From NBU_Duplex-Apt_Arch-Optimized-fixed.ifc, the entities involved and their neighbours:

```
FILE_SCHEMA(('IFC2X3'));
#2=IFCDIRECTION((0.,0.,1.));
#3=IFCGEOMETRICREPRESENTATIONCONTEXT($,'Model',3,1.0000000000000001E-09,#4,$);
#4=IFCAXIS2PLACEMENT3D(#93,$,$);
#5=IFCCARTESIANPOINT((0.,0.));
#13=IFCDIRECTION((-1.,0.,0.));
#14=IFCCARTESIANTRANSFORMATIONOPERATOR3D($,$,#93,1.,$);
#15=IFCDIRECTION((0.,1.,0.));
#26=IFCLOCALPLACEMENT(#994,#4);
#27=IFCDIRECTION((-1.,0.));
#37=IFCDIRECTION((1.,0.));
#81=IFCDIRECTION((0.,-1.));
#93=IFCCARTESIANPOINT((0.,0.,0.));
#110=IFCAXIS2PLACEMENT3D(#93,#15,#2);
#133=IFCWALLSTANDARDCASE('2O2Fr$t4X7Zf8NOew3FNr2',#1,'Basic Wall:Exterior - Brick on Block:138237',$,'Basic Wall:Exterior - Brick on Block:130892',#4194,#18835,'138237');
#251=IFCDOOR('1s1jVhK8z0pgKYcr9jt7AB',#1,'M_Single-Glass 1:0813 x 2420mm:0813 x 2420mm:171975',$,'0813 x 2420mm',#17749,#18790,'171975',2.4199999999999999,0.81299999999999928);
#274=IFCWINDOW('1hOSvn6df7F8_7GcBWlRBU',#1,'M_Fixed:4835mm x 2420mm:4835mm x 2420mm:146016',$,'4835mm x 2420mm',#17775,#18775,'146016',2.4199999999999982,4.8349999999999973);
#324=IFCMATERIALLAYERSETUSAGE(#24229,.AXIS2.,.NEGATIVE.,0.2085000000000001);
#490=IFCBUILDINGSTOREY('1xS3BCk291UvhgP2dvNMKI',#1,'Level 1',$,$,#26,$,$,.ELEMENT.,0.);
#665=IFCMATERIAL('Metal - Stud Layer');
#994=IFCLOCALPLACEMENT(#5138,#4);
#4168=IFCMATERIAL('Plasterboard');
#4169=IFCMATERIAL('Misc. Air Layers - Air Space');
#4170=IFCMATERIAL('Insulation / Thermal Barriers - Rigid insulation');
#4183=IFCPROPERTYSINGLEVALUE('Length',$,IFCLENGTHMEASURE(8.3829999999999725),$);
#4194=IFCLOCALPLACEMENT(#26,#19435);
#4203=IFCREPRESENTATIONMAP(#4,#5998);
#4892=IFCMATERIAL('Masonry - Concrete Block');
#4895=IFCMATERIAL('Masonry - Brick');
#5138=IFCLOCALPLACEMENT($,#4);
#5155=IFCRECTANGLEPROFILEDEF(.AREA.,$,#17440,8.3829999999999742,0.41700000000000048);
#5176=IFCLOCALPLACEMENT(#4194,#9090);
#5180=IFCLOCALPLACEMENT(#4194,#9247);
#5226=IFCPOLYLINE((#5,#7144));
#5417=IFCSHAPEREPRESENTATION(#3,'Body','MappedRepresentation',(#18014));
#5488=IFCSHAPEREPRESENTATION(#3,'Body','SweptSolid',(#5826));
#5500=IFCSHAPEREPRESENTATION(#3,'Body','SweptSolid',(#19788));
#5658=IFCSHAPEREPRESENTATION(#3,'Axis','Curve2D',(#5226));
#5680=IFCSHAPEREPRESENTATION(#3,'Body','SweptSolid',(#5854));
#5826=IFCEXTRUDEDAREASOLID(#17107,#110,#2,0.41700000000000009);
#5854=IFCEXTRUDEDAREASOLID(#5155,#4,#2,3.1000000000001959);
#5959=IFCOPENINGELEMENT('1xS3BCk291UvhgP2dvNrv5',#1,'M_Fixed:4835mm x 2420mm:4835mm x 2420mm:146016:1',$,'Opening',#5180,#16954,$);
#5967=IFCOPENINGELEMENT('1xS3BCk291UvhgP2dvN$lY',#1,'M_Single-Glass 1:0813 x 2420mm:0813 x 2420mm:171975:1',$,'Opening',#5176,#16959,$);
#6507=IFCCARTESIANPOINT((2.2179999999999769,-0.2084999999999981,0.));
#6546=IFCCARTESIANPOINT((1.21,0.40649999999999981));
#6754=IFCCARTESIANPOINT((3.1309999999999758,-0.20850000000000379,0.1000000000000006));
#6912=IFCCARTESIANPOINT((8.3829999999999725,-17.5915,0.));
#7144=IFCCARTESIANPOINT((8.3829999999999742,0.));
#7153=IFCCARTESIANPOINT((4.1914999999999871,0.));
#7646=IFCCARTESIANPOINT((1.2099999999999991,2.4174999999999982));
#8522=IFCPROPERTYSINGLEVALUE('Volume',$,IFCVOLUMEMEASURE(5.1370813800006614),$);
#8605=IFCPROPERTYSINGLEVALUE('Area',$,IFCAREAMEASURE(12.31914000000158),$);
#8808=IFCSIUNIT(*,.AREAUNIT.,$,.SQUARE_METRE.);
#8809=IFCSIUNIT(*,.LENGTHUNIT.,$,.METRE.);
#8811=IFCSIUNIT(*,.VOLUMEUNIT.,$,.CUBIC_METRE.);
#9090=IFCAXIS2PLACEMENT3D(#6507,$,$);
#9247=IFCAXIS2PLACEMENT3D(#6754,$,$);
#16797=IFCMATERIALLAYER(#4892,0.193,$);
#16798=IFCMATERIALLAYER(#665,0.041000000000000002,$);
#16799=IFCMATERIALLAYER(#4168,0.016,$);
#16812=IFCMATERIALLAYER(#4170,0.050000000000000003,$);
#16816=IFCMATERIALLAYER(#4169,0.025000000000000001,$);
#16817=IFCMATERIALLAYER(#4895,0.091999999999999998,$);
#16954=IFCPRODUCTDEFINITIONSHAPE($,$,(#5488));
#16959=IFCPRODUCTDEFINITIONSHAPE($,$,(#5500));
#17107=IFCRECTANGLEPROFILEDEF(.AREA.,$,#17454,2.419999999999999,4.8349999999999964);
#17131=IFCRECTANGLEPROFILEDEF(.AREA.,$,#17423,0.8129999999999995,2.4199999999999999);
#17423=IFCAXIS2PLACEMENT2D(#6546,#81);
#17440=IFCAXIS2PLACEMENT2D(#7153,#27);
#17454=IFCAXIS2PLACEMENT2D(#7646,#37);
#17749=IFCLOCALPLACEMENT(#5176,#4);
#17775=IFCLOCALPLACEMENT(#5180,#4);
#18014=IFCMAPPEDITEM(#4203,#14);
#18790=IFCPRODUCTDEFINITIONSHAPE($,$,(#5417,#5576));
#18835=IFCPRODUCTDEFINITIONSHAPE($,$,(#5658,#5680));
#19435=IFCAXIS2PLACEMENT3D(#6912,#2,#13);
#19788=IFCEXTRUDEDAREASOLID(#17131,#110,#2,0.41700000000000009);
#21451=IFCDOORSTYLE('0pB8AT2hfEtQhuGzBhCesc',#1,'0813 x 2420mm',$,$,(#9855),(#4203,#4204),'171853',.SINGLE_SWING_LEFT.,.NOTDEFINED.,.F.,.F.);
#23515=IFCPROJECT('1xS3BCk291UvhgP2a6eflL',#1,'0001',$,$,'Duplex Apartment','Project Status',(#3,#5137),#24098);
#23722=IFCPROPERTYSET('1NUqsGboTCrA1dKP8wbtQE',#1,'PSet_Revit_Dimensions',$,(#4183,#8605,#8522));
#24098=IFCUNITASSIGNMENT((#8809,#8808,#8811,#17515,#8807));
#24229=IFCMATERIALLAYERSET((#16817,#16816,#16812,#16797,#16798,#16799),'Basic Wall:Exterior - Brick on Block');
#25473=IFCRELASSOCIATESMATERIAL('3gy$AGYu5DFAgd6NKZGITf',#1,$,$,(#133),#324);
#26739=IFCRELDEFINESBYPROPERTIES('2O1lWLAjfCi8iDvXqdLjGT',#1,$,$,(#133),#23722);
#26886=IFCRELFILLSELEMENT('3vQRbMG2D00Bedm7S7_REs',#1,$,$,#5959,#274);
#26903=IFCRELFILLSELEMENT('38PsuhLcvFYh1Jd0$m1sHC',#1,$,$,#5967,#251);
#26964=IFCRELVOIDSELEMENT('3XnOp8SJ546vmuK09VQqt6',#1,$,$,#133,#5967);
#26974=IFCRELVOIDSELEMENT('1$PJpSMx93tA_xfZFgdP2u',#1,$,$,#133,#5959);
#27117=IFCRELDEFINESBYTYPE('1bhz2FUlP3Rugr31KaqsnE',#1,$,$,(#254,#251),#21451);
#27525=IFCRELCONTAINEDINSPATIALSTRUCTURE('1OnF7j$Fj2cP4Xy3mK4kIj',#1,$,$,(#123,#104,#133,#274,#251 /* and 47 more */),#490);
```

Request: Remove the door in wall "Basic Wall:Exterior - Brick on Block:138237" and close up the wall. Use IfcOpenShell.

```python
import ifcopenshell
import ifcopenshell.api.feature
import ifcopenshell.api.pset
import ifcopenshell.api.root
import ifcopenshell.geom
import ifcopenshell.util.element
import ifcopenshell.util.shape
import ifcopenshell.util.unit

model = ifcopenshell.open("NBU_Duplex-Apt_Arch-Optimized-fixed.ifc")
area_scale = ifcopenshell.util.unit.calculate_unit_scale(model, "AREAUNIT")
volume_scale = ifcopenshell.util.unit.calculate_unit_scale(model, "VOLUMEUNIT")
settings = ifcopenshell.geom.settings()


def volume(element):
    """Net volume in cubic metres, openings subtracted."""
    shape = ifcopenshell.geom.create_shape(settings, element)
    return ifcopenshell.util.shape.get_volume(shape.geometry)


door = model.by_guid("1s1jVhK8z0pgKYcr9jt7AB")
opening = door.FillsVoids[0].RelatingOpeningElement
wall = opening.VoidsElements[0].RelatingBuildingElement
before = volume(wall)

ifcopenshell.api.root.remove_product(model, product=door)
ifcopenshell.api.feature.remove_feature(model, feature=opening)

after = volume(wall)
thickness = 0.417  # wall thickness in metres

# Update the wall's stored quantities.
pset = model.by_id(ifcopenshell.util.element.get_pset(wall, "PSet_Revit_Dimensions", should_inherit=False)["id"])
ifcopenshell.api.pset.edit_pset(model, pset=pset, properties={
    "Area": model.create_entity("IfcAreaMeasure", after / thickness / area_scale),
    "Volume": model.create_entity("IfcVolumeMeasure", after / volume_scale),
})

print(f"wall volume {before:.3f} -> {after:.3f} m3")

model.write("NBU_Duplex-Apt_Arch-Optimized-fixed_rev.ifc")
```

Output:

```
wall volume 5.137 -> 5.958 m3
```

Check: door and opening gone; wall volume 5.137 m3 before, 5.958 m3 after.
